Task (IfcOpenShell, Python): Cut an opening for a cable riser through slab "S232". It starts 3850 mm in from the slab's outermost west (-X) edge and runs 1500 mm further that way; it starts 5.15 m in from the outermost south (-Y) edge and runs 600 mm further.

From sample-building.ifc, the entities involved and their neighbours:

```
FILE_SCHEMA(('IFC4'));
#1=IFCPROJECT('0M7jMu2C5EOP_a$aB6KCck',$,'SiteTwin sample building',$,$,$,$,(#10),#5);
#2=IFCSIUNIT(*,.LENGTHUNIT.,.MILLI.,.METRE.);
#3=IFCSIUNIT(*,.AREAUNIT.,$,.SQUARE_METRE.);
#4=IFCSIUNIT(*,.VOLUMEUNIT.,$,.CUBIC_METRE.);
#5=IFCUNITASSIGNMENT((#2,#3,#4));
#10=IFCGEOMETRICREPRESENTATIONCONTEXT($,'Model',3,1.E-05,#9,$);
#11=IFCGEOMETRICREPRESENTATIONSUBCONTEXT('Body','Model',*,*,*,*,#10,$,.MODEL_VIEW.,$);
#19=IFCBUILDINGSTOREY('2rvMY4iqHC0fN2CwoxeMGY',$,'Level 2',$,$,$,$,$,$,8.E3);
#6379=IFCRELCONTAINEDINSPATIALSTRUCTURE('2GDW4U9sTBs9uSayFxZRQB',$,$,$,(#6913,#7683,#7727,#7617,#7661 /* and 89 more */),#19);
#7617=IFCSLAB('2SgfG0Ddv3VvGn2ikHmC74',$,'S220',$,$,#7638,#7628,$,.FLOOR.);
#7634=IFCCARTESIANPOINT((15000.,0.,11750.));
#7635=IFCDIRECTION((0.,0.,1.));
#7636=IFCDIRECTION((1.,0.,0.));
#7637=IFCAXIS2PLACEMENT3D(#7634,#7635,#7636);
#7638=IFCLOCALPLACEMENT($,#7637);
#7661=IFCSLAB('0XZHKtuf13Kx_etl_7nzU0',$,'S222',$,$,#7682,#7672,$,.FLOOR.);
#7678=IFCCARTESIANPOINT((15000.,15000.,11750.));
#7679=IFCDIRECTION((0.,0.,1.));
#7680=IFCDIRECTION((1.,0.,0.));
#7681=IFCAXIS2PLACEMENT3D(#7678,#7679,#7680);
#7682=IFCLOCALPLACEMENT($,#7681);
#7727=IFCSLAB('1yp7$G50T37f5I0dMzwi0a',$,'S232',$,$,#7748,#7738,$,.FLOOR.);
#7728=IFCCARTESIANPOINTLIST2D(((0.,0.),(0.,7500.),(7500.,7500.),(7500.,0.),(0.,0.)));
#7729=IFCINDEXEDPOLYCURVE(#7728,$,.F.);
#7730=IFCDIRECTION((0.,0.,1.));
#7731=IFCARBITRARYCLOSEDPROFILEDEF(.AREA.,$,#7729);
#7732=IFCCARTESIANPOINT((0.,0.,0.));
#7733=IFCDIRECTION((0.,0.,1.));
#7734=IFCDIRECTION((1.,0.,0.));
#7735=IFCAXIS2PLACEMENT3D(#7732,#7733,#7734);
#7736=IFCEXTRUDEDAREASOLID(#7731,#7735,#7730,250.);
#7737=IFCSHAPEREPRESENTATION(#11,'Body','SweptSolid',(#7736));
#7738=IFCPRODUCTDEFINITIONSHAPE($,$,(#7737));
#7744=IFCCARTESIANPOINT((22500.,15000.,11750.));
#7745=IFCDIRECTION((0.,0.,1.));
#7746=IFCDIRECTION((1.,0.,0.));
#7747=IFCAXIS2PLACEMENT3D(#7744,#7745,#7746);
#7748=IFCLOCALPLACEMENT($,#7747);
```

```python
import numpy as np
import ifcopenshell
import ifcopenshell.api.feature
import ifcopenshell.api.geometry
import ifcopenshell.api.root
import ifcopenshell.geom
import ifcopenshell.util.placement
import ifcopenshell.util.representation
import ifcopenshell.util.shape
import ifcopenshell.util.unit

model = ifcopenshell.open("sample-building.ifc")
unit_scale = ifcopenshell.util.unit.calculate_unit_scale(model)
settings = ifcopenshell.geom.settings()


def volume(element):
    """Net volume in cubic metres, openings subtracted."""
    shape = ifcopenshell.geom.create_shape(settings, element)
    return ifcopenshell.util.shape.get_volume(shape.geometry)


slab = model.by_id(7727)
before = volume(slab)

# Extent in the slab's own axes, in metres. The edges named are its -X and -Y sides.
slab_shape = ifcopenshell.geom.create_shape(settings, slab)
vertices = ifcopenshell.util.shape.get_vertices(slab_shape.geometry)
x_min, y_min, bottom = vertices.min(axis=0)
top = vertices[:, 2].max()

opening = ifcopenshell.api.root.create_entity(model, ifc_class="IfcOpeningElement", name="Cable riser opening", predefined_type="OPENING")
context = ifcopenshell.util.representation.get_context(model, "Model", "Body", "MODEL_VIEW")
width, depth = 1.5, 0.6
outline = [(0.0, 0.0), (width, 0.0), (width, depth), (0.0, depth), (0.0, 0.0)]
# Overshoot both faces by 50 mm so the cut is clean.
shape = ifcopenshell.api.geometry.add_slab_representation(
    model, context=context, depth=top - bottom + 0.1, polyline=outline
)
ifcopenshell.api.geometry.assign_representation(model, product=opening, representation=shape)

matrix = ifcopenshell.util.placement.get_local_placement(slab.ObjectPlacement)
matrix[:, 3] = matrix @ np.append(np.array([x_min + 3.85, y_min + 5.15, bottom - 0.05]) / unit_scale, 1.0)
ifcopenshell.api.geometry.edit_object_placement(model, product=opening, matrix=matrix, is_si=False)
ifcopenshell.api.feature.add_feature(model, feature=opening, element=slab)

after = volume(slab)

print(f"slab volume {before:.3f} -> {after:.3f} m3")

model.write("sample-building_rev.ifc")
```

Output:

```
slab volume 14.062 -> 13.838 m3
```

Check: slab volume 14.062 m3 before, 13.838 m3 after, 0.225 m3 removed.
